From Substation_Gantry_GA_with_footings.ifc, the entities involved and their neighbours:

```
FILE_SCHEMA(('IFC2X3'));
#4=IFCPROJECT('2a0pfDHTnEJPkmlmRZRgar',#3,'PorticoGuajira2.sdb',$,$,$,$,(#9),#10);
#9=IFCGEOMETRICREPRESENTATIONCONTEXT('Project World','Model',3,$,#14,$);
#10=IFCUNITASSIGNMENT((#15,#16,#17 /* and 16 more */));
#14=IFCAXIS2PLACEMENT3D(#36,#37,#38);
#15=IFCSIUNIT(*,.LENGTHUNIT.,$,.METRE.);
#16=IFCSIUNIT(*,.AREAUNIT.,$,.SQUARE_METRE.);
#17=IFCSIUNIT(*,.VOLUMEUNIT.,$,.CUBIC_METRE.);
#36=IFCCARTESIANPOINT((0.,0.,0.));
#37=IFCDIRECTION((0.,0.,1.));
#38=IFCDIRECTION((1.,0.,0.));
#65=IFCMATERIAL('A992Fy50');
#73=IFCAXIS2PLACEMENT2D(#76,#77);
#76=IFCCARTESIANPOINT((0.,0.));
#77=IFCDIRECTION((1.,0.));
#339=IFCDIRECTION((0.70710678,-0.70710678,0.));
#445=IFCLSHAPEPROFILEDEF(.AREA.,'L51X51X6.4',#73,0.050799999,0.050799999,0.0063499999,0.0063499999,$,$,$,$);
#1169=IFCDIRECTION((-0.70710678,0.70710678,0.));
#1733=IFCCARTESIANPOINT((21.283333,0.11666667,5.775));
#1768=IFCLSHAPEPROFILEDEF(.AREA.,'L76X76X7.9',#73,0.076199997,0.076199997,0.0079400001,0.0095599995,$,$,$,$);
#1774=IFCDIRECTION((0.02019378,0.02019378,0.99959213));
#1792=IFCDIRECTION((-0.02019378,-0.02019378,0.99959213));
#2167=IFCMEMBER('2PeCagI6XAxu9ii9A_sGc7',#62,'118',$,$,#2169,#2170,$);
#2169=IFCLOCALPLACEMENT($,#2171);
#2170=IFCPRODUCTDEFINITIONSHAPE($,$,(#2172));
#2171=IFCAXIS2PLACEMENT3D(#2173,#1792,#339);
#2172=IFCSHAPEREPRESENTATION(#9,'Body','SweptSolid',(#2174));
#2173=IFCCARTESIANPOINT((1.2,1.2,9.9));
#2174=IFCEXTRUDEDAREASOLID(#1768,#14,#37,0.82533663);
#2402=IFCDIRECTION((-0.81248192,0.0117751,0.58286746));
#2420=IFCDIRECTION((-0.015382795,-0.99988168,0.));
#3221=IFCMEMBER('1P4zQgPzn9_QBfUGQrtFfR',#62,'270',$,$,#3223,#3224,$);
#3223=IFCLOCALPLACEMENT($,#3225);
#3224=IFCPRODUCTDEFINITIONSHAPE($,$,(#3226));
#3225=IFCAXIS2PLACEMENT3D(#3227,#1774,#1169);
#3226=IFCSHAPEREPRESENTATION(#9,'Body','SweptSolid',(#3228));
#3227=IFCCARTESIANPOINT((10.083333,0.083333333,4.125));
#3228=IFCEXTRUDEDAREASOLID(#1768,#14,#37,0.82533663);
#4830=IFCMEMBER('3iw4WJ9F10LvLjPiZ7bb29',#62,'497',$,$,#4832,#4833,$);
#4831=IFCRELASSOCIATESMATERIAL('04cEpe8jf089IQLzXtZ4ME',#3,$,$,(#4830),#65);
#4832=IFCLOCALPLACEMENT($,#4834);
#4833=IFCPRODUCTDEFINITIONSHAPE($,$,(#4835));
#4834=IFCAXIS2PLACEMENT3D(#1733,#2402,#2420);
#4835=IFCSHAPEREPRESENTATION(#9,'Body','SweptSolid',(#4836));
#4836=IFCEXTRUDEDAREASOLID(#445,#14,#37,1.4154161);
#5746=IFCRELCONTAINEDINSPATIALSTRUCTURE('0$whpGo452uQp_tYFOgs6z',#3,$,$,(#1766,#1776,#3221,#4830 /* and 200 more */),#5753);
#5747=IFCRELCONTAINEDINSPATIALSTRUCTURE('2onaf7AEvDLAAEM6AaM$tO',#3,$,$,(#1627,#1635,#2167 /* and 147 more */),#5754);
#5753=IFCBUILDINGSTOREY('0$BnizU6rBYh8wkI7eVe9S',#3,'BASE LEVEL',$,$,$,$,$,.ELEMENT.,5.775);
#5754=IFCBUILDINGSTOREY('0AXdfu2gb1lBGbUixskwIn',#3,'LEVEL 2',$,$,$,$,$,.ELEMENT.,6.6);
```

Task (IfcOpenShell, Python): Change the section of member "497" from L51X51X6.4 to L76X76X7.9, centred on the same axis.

```python
import ifcopenshell
import ifcopenshell.util.element

model = ifcopenshell.open("Substation_Gantry_GA_with_footings.ifc")

member = model.by_guid("3iw4WJ9F10LvLjPiZ7bb29")
source = next(p for p in model.by_type("IfcLShapeProfileDef") if p.ProfileName == "L76X76X7.9")

body = next(r for r in member.Representation.Representations if r.RepresentationIdentifier == "Body")
solid = body.Items[0]
old_profile = solid.SweptArea

# Copy the section's sizes but keep this member's own profile position.
profile = ifcopenshell.util.element.copy(model, source)
profile.Position = old_profile.Position
solid.SweptArea = profile
if not model.get_total_inverses(old_profile):
    ifcopenshell.util.element.remove_deep2(model, old_profile)

print(solid.SweptArea)

model.write("Substation_Gantry_GA_with_footings_v2.ifc")
```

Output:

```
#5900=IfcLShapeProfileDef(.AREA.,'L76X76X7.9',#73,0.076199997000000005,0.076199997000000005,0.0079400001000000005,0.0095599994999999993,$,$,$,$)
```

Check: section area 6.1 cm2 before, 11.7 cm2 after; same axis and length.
